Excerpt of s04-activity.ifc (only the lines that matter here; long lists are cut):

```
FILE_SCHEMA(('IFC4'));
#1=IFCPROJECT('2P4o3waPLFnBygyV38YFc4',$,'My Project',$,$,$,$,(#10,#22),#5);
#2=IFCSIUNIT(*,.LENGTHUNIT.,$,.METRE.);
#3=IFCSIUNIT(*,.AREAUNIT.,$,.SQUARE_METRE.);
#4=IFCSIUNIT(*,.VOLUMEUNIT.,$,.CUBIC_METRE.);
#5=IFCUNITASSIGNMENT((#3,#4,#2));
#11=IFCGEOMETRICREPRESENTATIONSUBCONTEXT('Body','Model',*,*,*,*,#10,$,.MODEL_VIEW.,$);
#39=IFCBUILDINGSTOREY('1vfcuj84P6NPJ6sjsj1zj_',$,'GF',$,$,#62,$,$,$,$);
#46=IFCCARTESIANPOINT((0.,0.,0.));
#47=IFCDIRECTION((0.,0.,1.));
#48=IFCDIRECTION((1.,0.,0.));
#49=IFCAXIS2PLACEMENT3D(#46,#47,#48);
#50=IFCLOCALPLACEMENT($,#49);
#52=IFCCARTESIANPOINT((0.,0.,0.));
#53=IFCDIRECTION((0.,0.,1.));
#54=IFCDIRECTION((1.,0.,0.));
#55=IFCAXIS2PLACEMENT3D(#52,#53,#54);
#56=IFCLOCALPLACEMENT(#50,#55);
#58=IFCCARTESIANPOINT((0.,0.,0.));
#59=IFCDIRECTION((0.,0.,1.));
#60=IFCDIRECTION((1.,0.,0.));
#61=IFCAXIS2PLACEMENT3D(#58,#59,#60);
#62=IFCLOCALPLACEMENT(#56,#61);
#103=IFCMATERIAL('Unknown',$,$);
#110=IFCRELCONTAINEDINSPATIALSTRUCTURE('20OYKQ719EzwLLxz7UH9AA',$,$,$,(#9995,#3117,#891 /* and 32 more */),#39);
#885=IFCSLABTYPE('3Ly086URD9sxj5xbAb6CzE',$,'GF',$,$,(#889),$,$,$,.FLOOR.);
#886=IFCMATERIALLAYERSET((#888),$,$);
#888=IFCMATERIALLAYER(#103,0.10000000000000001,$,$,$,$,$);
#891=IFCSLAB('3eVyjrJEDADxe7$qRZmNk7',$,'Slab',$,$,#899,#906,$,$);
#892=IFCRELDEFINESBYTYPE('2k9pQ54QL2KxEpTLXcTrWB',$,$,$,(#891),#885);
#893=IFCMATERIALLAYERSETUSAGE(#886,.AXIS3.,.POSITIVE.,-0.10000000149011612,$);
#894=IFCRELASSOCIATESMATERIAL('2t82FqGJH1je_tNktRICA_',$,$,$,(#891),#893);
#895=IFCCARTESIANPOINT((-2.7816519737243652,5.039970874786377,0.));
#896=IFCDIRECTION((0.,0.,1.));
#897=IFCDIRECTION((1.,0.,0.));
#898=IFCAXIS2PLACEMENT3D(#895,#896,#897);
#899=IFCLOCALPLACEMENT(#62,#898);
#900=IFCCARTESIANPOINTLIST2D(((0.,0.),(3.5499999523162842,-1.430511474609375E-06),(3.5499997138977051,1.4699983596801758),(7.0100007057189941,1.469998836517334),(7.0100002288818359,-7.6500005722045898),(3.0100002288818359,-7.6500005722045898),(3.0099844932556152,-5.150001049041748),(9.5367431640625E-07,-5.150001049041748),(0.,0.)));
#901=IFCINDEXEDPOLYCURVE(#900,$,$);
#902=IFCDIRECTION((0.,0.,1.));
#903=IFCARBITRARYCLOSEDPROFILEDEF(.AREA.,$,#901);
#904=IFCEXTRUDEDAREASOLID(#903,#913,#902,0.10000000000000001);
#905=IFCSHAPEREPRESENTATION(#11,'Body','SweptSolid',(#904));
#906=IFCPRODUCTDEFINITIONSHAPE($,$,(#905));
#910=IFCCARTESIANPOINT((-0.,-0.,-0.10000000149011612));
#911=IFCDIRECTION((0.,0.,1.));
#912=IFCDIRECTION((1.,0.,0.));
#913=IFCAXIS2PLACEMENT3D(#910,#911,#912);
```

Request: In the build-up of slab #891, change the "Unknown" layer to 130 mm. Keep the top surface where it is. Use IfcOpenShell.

```python
import ifcopenshell
import ifcopenshell.util.element
import ifcopenshell.util.representation
import ifcopenshell.util.unit

model = ifcopenshell.open("s04-activity.ifc")
unit_scale = ifcopenshell.util.unit.calculate_unit_scale(model)

layer_set = model.by_id(886)
layer = next(l for l in layer_set.MaterialLayers if l.Material and l.Material.Name == "Unknown")
change = 0.13 / unit_scale - layer.LayerThickness
layer.LayerThickness += change

# Geometry does not follow the layer set by itself.
slabs = [e for e in ifcopenshell.util.element.get_elements_by_material(model, layer_set) if e.is_a("IfcSlab")]
for slab in sorted(slabs, key=lambda e: e.id()):
    body = ifcopenshell.util.representation.get_representation(slab, "Model", "Body")
    solid = body.Items[0]
    old_depth = solid.Depth
    solid.Depth += change
    # Extruded upwards: lower the start of the extrusion so the top stays.
    x, y, z = solid.Position.Location.Coordinates
    solid.Position.Location = model.createIfcCartesianPoint((x, y, z - change))
    print(slab.id(), f"{old_depth:g} -> {solid.Depth:g}")

# The layers are counted up from the underside, which has moved.
for usage in {ifcopenshell.util.element.get_material(slab) for slab in slabs}:
    usage.OffsetFromReferenceLine -= change

model.write("s04-activity-out.ifc")
```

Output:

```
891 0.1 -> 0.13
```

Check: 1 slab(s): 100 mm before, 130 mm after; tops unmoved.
